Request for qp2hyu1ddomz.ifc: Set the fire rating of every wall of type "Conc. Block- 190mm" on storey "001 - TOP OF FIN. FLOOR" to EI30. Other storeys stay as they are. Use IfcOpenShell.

First a look at what the model holds.

```python
import ifcopenshell
import ifcopenshell.util.element

model = ifcopenshell.open("qp2hyu1ddomz.ifc")
print(model.schema)
storey = next(s for s in model.by_type("IfcBuildingStorey") if s.Name == "001 - TOP OF FIN. FLOOR")
walls = [e for e in ifcopenshell.util.element.get_decomposition(storey) if e.is_a("IfcWall")]
seen = {}
for e in walls:
    element_type = ifcopenshell.util.element.get_type(e)
    key = (element_type.Name if element_type != e and element_type else None, ifcopenshell.util.element.get_pset(e, "Pset_WallCommon", "FireRating"))
    seen[key] = seen.get(key, 0) + 1
for (name, value), count in sorted(seen.items(), key=str):
    print(count, "x", name, "|", value)
```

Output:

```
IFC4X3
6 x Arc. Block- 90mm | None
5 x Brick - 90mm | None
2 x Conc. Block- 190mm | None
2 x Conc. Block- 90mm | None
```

```python
import ifcopenshell
import ifcopenshell.api.pset
import ifcopenshell.util.element

model = ifcopenshell.open("qp2hyu1ddomz.ifc")

storey = next(s for s in model.by_type("IfcBuildingStorey") if s.Name == "001 - TOP OF FIN. FLOOR")
walls = [e for e in ifcopenshell.util.element.get_decomposition(storey) if e.is_a("IfcWall")]

count = 0
for e in walls:
    element_type = ifcopenshell.util.element.get_type(e)
    if element_type in (None, e) or element_type.Name != "Conc. Block- 190mm":
        continue
    # add_pset returns the element's existing set when there is one.
    pset = ifcopenshell.api.pset.add_pset(model, product=e, name="Pset_WallCommon")
    ifcopenshell.api.pset.edit_pset(model, pset=pset, properties={"FireRating": "EI30"})
    count += 1

print(count, "walls updated")

model.write("qp2hyu1ddomz-out.ifc")
```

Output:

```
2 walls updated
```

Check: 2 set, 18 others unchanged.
